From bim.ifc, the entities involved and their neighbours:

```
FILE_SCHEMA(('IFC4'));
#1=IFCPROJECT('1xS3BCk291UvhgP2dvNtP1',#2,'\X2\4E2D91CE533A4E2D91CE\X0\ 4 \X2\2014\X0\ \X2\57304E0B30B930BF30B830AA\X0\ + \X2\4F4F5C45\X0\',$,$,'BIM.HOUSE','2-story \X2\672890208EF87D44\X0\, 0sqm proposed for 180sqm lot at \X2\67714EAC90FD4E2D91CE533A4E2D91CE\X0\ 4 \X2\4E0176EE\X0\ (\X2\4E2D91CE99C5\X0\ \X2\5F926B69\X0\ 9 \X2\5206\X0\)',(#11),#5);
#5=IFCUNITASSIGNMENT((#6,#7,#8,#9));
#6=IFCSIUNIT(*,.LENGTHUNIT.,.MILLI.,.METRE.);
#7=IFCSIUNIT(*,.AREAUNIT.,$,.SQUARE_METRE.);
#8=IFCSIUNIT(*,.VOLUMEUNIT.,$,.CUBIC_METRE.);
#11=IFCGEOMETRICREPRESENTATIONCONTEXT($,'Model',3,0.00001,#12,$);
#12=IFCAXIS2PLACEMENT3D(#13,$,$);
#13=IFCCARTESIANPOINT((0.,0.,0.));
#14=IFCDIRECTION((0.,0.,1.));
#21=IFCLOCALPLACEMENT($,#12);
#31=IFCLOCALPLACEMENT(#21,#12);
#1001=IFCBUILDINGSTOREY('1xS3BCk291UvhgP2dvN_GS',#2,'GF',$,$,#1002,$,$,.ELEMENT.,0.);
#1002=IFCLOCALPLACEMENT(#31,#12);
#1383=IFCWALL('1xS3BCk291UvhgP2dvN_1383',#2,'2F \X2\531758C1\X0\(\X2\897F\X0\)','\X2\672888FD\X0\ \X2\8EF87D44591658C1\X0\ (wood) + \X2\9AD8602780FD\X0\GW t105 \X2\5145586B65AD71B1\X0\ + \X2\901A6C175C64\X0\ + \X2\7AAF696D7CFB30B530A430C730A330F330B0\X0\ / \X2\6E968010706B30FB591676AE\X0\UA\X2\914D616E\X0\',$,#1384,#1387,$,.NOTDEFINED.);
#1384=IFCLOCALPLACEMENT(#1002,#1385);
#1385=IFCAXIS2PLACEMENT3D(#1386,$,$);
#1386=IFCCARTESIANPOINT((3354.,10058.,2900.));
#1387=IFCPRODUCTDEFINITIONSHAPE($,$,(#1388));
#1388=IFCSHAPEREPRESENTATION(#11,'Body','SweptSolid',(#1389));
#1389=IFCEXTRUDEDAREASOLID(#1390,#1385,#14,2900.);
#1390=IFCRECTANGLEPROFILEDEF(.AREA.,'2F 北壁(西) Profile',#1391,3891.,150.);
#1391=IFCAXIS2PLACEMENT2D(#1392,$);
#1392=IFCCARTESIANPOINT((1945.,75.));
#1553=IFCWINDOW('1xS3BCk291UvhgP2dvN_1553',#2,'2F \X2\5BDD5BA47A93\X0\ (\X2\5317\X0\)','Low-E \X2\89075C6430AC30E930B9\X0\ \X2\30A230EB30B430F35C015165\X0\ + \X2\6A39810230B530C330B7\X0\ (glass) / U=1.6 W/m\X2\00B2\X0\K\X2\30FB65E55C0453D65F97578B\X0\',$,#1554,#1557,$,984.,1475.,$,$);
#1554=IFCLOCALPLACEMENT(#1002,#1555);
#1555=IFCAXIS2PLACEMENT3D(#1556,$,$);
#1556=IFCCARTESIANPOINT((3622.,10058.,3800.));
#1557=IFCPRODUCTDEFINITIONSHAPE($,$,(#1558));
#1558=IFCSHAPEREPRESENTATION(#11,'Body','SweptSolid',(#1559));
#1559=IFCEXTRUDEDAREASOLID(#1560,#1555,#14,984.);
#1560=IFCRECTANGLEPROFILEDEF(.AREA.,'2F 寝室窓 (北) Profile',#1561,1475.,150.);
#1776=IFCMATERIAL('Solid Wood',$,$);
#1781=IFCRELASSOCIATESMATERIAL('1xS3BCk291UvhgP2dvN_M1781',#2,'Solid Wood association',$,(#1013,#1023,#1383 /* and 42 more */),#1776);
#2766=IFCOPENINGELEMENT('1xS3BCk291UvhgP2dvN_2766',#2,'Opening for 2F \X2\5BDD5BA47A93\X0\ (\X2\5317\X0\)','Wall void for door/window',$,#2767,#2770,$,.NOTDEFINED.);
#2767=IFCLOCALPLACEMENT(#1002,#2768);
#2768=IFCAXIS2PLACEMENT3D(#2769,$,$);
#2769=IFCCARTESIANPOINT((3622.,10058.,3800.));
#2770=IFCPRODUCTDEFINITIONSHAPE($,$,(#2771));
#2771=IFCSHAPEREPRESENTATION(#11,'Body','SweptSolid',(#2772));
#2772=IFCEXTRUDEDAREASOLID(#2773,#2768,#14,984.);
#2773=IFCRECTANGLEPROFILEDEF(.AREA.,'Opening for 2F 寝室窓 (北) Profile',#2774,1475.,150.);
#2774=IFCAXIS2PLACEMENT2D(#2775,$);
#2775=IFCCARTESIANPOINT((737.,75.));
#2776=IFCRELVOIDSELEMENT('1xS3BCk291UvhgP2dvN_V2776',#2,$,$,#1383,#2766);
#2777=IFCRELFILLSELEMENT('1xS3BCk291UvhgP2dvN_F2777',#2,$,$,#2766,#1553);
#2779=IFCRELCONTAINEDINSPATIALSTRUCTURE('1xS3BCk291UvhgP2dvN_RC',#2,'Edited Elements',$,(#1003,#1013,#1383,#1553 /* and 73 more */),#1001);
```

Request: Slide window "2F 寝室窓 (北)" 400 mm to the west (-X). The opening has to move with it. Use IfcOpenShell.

```python
import ifcopenshell
import ifcopenshell.api.geometry
import ifcopenshell.util.placement
import ifcopenshell.util.unit

model = ifcopenshell.open("bim.ifc")
unit_scale = ifcopenshell.util.unit.calculate_unit_scale(model)

window = model.by_guid("1xS3BCk291UvhgP2dvN_1553")
opening = window.FillsVoids[0].RelatingOpeningElement
wall = opening.VoidsElements[0].RelatingBuildingElement

wall_matrix = ifcopenshell.util.placement.get_local_placement(wall.ObjectPlacement)
shift = wall_matrix[:3, 0] * -0.4 / unit_scale
before = ifcopenshell.util.placement.get_local_placement(window.ObjectPlacement)[:3, 3].copy()

# The window is not placed relative to its opening, so move both.
for product in (opening, window):
    matrix = ifcopenshell.util.placement.get_local_placement(product.ObjectPlacement)
    matrix[:3, 3] += shift
    ifcopenshell.api.geometry.edit_object_placement(model, product=product, matrix=matrix, is_si=False)

after = ifcopenshell.util.placement.get_local_placement(window.ObjectPlacement)[:3, 3]
print("window moved by", (after - before).round(3) + 0.0)

model.write("bim_v2.ifc")
```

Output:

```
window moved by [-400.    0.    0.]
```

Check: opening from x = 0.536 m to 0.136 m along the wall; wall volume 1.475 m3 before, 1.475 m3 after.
